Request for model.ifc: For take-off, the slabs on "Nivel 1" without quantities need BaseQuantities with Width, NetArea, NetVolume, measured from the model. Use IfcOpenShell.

First a look at what the model holds.

```python
import ifcopenshell
import ifcopenshell.util.element
import ifcopenshell.util.unit

model = ifcopenshell.open("model.ifc")
print(model.schema)
for unit_type in ("LENGTHUNIT", "AREAUNIT", "VOLUMEUNIT"):
    print(unit_type, ifcopenshell.util.unit.calculate_unit_scale(model, unit_type))
storey = next(s for s in model.by_type("IfcBuildingStorey") if s.Name == "Nivel 1")
slabs = [e for e in ifcopenshell.util.element.get_decomposition(storey) if e.is_a("IfcSlab")]
for e in sorted(slabs, key=lambda e: e.id()):
    print(e.id(), e.is_a(), e.Name, list(ifcopenshell.util.element.get_psets(e, qtos_only=True)), sep=" | ")
```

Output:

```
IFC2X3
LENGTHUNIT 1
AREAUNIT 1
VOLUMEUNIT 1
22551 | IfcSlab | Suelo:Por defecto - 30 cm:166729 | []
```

```python
import ifcopenshell
import ifcopenshell.api.pset
import ifcopenshell.geom
import ifcopenshell.util.element
import ifcopenshell.util.shape
import ifcopenshell.util.unit

model = ifcopenshell.open("model.ifc")
unit_scale = ifcopenshell.util.unit.calculate_unit_scale(model)
area_scale = ifcopenshell.util.unit.calculate_unit_scale(model, "AREAUNIT")
volume_scale = ifcopenshell.util.unit.calculate_unit_scale(model, "VOLUMEUNIT")
settings = ifcopenshell.geom.settings()

storey = next(s for s in model.by_type("IfcBuildingStorey") if s.Name == "Nivel 1")
slabs = [e for e in ifcopenshell.util.element.get_decomposition(storey) if e.is_a("IfcSlab")]

for e in sorted(slabs, key=lambda e: e.id()):
    if ifcopenshell.util.element.get_psets(e, qtos_only=True, should_inherit=False):
        continue
    # Geometry comes back in metres, in the element's own axes.
    shape = ifcopenshell.geom.create_shape(settings, e)
    values = {
        "Width": ifcopenshell.util.shape.get_z(shape.geometry) / unit_scale,
        "NetArea": ifcopenshell.util.shape.get_footprint_area(shape.geometry) / area_scale,
        "NetVolume": ifcopenshell.util.shape.get_volume(shape.geometry) / volume_scale,
    }
    qto = ifcopenshell.api.pset.add_qto(model, product=e, name="BaseQuantities")
    ifcopenshell.api.pset.edit_qto(model, qto=qto, properties=values)
    print(e.id(), {k: round(v, 3) for k, v in values.items()})

model.write("model-out.ifc")
```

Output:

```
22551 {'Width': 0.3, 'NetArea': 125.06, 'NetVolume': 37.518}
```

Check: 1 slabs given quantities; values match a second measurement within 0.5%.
